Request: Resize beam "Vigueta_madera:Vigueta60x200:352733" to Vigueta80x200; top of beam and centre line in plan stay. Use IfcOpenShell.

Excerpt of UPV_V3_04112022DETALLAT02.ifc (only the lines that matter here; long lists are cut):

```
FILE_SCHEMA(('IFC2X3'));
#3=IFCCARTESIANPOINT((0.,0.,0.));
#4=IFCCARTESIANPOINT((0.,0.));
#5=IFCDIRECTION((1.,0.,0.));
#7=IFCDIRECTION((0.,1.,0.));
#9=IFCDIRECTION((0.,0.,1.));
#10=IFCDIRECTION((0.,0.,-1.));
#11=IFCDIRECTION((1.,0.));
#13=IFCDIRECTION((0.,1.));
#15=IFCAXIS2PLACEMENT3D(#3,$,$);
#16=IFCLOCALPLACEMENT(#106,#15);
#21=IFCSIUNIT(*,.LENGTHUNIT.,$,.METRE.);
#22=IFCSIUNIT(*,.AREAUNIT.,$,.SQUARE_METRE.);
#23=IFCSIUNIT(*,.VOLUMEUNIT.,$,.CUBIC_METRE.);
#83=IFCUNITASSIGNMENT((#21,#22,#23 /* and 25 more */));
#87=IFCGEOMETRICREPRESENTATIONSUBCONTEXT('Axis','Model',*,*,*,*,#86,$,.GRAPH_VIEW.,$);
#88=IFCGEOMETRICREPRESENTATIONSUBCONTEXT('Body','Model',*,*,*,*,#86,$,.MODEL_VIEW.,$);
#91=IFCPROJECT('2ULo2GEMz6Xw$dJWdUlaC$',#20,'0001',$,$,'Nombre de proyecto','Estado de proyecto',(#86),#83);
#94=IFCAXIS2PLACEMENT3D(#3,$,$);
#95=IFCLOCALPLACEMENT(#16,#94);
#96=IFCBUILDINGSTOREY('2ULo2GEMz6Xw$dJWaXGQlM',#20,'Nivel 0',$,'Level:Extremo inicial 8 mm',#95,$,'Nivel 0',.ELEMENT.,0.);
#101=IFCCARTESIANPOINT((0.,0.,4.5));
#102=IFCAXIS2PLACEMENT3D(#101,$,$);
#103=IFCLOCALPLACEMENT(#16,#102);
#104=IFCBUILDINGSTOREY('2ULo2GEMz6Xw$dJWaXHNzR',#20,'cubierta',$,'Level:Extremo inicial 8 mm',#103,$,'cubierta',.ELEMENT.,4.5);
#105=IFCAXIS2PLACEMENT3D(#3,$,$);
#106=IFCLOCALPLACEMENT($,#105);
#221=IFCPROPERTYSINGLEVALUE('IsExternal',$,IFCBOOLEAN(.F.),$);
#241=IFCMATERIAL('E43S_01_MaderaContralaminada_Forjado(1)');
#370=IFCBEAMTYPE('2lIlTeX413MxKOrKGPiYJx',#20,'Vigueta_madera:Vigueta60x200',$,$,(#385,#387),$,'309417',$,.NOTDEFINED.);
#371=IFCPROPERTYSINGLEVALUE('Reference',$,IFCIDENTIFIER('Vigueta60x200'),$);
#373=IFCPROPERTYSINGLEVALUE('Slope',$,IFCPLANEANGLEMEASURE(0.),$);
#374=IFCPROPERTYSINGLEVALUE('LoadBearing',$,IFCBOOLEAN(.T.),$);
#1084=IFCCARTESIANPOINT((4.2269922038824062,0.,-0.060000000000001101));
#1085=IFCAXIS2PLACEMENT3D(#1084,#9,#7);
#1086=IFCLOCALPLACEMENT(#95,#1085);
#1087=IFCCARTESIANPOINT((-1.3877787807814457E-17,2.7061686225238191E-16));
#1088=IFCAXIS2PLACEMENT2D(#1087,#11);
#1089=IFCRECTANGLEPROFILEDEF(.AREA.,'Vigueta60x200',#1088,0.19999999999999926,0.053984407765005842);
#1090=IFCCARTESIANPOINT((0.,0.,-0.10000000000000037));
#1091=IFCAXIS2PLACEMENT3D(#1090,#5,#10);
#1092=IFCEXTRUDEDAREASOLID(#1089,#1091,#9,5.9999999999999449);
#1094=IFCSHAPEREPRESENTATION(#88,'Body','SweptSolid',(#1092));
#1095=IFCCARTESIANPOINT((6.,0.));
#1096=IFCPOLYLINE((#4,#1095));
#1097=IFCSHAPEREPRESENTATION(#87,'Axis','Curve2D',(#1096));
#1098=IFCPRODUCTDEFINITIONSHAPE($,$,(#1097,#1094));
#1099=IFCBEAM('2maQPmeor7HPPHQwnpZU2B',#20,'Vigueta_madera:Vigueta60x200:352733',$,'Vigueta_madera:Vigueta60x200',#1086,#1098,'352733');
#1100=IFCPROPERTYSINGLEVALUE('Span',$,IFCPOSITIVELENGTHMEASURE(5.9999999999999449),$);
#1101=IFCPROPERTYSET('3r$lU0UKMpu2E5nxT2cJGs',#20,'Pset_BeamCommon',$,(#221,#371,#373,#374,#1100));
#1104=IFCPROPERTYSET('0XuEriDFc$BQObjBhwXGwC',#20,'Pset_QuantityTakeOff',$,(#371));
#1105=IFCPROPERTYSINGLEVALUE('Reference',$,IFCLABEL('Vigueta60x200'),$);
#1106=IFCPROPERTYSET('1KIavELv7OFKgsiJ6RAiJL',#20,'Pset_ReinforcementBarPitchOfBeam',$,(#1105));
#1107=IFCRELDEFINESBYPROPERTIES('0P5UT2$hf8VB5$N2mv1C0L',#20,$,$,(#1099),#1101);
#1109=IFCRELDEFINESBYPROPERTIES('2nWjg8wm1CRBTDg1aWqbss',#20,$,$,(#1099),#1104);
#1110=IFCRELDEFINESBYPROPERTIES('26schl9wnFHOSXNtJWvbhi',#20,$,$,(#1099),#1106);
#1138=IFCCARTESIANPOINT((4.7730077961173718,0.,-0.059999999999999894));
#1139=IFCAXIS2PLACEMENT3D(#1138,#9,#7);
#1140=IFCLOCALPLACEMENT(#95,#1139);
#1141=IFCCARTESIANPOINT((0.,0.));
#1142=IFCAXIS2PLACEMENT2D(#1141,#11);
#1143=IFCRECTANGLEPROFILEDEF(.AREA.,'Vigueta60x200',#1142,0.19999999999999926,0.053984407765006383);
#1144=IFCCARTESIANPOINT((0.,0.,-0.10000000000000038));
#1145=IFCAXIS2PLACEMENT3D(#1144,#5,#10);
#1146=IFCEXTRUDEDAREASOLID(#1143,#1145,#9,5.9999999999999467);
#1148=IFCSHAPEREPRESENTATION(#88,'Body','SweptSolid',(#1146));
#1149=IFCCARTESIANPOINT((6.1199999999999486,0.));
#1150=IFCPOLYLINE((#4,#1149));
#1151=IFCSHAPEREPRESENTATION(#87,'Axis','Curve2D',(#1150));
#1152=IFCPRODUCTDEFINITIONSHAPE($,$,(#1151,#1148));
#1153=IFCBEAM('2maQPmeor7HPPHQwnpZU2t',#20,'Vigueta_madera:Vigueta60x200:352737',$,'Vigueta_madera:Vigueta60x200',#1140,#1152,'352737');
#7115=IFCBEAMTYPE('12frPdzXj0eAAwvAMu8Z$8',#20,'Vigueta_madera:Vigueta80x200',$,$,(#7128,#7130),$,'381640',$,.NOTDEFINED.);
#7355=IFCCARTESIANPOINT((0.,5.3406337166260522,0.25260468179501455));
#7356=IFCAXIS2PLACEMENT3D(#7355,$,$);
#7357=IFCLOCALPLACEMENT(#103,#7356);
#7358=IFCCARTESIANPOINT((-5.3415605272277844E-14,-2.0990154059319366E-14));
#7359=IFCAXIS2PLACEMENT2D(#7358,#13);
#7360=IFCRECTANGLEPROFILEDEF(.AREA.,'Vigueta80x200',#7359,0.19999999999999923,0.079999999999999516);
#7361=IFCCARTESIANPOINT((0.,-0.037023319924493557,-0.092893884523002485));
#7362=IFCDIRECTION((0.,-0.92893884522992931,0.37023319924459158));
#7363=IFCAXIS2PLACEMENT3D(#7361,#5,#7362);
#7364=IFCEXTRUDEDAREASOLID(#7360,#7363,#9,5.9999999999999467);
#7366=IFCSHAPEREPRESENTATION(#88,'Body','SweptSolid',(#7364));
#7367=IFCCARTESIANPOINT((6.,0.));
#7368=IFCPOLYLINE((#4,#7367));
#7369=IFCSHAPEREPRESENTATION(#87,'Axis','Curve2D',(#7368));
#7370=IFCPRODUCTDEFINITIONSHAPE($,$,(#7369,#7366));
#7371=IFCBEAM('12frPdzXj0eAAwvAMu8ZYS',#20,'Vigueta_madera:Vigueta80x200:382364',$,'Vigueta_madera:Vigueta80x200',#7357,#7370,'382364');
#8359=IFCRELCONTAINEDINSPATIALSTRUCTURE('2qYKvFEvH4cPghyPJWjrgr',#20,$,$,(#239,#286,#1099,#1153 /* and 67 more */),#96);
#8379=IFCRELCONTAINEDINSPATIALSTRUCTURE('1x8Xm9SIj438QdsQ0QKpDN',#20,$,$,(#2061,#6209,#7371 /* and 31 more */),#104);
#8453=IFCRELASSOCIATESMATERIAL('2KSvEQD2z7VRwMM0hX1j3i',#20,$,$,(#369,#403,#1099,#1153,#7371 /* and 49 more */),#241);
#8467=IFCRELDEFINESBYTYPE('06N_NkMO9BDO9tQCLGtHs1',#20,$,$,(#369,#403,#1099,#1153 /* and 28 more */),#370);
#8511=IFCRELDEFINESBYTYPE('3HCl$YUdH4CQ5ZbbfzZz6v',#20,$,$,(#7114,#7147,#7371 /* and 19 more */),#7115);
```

```python
import ifcopenshell
import ifcopenshell.api.pset
import ifcopenshell.api.type
import ifcopenshell.util.element
import ifcopenshell.util.representation

model = ifcopenshell.open("UPV_V3_04112022DETALLAT02.ifc")

member = model.by_guid("2maQPmeor7HPPHQwnpZU2B")
source = next(p for p in model.by_type("IfcRectangleProfileDef") if p.ProfileName == "Vigueta80x200")

body = ifcopenshell.util.representation.get_representation(member, "Model", "Body")
solid = body.Items[0]
old_profile = solid.SweptArea

# Copy the section's sizes but keep this member's own profile position.
profile = ifcopenshell.util.element.copy(model, source)
# Profiles are centred, so shift by half the change in depth to hold the top.
shift = (old_profile.XDim - profile.XDim) / 2
x, y = old_profile.Position.Location.Coordinates
up = (-1.0, 0.0)  # upwards, in the solid's own plane
location = model.createIfcCartesianPoint((x + up[0] * shift, y + up[1] * shift))
profile.Position = model.createIfcAxis2Placement2D(location, old_profile.Position.RefDirection)
solid.SweptArea = profile
if not model.get_total_inverses(old_profile):
    ifcopenshell.util.element.remove_deep2(model, old_profile)

new_type = model.by_id(7115)
ifcopenshell.api.type.assign_type(
    model, related_objects=[member], relating_type=new_type, should_map_representations=False
)
member.Name = member.Name.replace("Vigueta60x200", "Vigueta80x200")
member.ObjectType = "Vigueta_madera:Vigueta80x200"
pset = model.by_id(ifcopenshell.util.element.get_pset(member, "Pset_BeamCommon", should_inherit=False)["id"])
ifcopenshell.api.pset.edit_pset(model, pset=pset, properties={"Reference": "Vigueta80x200"})
pset = model.by_id(ifcopenshell.util.element.get_pset(member, "Pset_QuantityTakeOff", should_inherit=False)["id"])
ifcopenshell.api.pset.edit_pset(model, pset=pset, properties={"Reference": "Vigueta80x200"})
pset = model.by_id(ifcopenshell.util.element.get_pset(member, "Pset_ReinforcementBarPitchOfBeam", should_inherit=False)["id"])
ifcopenshell.api.pset.edit_pset(model, pset=pset, properties={"Reference": "Vigueta80x200"})

print(solid.SweptArea)

model.write("UPV_V3_04112022DETALLAT02_updated.ifc")
```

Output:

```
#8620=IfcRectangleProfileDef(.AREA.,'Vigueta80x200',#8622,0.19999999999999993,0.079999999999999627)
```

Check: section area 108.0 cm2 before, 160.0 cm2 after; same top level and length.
